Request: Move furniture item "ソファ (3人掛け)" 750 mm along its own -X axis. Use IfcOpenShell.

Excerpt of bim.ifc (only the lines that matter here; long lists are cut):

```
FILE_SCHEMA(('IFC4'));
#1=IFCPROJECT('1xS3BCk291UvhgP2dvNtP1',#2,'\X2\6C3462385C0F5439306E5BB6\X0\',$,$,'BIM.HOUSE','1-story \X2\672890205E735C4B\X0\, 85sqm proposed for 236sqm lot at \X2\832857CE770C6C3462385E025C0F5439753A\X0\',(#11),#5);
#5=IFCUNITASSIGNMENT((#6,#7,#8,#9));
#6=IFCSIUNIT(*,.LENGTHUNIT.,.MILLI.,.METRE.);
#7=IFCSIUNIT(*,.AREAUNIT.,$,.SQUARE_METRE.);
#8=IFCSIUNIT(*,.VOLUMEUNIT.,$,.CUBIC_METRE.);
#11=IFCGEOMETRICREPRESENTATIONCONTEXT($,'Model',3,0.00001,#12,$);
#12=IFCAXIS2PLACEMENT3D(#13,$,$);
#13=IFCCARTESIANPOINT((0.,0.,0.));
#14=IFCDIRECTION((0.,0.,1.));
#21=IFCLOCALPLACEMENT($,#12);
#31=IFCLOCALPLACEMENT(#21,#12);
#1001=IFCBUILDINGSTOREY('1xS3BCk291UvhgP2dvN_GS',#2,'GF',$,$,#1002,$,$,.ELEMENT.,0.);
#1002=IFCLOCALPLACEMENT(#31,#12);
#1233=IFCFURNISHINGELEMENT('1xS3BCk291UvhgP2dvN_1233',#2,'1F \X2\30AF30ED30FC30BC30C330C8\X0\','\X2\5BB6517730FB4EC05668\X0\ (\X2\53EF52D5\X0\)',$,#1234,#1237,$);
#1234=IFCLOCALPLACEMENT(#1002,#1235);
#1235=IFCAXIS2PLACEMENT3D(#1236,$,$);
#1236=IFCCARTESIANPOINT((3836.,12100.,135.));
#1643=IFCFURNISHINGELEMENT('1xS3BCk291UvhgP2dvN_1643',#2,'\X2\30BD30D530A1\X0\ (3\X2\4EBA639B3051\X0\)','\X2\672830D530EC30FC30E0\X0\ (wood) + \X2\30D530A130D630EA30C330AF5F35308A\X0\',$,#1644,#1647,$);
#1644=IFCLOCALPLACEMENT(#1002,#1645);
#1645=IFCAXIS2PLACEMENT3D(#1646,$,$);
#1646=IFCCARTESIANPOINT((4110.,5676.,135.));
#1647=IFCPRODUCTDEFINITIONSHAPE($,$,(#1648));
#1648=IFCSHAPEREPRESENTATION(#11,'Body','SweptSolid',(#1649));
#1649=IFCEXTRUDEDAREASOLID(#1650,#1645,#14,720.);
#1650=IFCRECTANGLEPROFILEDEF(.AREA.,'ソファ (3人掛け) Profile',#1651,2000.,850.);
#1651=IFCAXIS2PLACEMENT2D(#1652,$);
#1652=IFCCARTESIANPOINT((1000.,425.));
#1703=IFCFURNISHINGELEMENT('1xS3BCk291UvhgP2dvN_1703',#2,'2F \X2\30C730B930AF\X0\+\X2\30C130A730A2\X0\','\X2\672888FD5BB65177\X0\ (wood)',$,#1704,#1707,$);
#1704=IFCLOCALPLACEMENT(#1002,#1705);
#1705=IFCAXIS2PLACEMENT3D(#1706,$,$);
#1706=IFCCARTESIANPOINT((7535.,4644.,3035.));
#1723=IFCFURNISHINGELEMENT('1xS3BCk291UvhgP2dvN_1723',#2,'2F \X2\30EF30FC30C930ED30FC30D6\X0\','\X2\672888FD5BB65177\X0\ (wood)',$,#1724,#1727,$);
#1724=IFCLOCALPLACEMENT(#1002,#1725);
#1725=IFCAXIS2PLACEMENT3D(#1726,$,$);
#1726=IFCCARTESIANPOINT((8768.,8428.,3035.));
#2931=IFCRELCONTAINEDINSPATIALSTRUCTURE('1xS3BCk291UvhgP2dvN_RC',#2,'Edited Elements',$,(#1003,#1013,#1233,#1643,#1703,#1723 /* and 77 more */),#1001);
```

```python
import ifcopenshell
import ifcopenshell.api.geometry
import ifcopenshell.util.placement
import ifcopenshell.util.unit

model = ifcopenshell.open("bim.ifc")
unit_scale = ifcopenshell.util.unit.calculate_unit_scale(model)

item = model.by_guid("1xS3BCk291UvhgP2dvN_1643")
matrix = ifcopenshell.util.placement.get_local_placement(item.ObjectPlacement)
matrix[:3, 3] -= matrix[:3, 0] * 0.75 / unit_scale
ifcopenshell.api.geometry.edit_object_placement(model, product=item, matrix=matrix, is_si=False)

print(ifcopenshell.util.placement.get_local_placement(item.ObjectPlacement).round(3) + 0.0)

model.write("bim_edited.ifc")
```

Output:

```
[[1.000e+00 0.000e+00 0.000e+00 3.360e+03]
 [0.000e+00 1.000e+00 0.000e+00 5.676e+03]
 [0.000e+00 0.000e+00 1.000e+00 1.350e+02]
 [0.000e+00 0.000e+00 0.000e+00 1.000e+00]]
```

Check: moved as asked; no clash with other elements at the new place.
